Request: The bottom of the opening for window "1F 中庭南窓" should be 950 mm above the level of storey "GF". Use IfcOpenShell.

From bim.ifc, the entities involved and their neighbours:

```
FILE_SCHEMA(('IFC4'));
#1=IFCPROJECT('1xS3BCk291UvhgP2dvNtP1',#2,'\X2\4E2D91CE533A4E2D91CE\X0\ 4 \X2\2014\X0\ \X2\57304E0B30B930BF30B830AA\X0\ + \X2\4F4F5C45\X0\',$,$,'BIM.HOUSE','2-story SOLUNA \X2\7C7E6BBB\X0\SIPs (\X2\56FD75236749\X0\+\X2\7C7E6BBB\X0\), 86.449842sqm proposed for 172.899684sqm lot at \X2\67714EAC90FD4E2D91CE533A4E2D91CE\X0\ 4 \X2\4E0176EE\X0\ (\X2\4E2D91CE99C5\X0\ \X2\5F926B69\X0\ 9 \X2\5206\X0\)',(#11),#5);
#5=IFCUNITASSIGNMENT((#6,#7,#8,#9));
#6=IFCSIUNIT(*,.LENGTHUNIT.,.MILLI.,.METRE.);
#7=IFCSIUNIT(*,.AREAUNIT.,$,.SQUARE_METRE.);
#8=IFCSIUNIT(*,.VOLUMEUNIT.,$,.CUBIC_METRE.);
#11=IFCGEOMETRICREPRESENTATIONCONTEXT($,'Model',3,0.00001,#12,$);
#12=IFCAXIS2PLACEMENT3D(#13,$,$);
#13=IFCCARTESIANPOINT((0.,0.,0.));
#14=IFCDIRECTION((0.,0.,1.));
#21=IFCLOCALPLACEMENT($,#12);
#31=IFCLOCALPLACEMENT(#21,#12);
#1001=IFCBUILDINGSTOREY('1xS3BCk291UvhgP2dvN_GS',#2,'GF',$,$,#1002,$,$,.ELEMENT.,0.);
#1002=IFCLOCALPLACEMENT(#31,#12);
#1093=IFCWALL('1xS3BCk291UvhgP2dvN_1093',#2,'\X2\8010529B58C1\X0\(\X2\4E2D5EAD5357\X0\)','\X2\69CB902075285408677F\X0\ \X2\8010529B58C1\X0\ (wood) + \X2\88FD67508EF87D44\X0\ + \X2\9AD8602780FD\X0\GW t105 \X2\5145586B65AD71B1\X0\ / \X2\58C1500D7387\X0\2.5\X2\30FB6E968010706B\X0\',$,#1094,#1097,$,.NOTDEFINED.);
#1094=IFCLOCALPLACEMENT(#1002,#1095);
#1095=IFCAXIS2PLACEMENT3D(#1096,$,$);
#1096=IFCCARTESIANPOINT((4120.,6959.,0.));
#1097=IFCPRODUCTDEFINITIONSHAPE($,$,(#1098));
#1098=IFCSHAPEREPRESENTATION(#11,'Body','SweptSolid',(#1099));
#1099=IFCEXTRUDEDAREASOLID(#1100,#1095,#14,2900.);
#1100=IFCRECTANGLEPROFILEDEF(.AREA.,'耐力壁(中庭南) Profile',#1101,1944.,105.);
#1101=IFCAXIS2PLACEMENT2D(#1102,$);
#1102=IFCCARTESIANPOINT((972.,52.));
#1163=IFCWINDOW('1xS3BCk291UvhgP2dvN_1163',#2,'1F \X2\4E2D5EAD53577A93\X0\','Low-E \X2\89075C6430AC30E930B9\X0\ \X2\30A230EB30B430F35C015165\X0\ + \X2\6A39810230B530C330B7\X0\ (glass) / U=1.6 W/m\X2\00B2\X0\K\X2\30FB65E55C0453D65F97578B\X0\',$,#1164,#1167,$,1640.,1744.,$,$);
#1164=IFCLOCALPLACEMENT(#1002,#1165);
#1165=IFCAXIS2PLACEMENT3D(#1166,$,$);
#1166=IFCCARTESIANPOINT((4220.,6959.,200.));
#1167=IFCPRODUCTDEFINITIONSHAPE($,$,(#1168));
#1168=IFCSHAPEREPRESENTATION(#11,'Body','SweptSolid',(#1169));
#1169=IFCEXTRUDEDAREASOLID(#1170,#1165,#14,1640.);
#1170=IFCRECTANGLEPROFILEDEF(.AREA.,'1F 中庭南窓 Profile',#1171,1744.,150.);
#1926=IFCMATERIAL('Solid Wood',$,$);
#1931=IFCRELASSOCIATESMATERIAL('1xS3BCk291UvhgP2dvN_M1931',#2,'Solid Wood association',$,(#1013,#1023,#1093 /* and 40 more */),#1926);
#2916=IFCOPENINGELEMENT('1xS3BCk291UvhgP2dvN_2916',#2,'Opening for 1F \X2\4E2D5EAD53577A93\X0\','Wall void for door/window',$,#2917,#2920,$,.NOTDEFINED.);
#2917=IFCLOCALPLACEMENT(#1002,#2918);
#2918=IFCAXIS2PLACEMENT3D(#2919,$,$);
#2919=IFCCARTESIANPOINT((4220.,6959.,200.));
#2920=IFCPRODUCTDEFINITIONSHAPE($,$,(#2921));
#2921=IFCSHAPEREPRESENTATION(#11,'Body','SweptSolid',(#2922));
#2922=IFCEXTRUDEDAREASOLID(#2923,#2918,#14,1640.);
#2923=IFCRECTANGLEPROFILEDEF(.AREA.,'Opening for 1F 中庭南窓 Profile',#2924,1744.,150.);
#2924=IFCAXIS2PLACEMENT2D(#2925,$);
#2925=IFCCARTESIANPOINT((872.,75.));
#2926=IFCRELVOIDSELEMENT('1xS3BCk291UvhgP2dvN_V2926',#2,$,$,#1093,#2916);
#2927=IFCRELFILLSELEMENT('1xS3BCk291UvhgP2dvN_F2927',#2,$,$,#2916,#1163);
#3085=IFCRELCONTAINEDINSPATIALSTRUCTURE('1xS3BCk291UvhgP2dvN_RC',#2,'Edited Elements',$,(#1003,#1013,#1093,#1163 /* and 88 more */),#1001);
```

```python
import numpy as np
import ifcopenshell
import ifcopenshell.api.geometry
import ifcopenshell.geom
import ifcopenshell.util.element
import ifcopenshell.util.placement
import ifcopenshell.util.shape
import ifcopenshell.util.unit

model = ifcopenshell.open("bim.ifc")
unit_scale = ifcopenshell.util.unit.calculate_unit_scale(model)

window = model.by_guid("1xS3BCk291UvhgP2dvN_1163")
opening = window.FillsVoids[0].RelatingOpeningElement
storey = ifcopenshell.util.element.get_container(window, ifc_class="IfcBuildingStorey")
level = ifcopenshell.util.placement.get_local_placement(storey.ObjectPlacement)[2, 3]

# The opening's origin need not be at the sill, so measure its lowest point.
shape = ifcopenshell.geom.create_shape(ifcopenshell.geom.settings(), opening)
bottom = ifcopenshell.util.shape.get_shape_bottom_elevation(shape, shape.geometry) / unit_scale
dz = level + 0.95 / unit_scale - bottom

shift = np.array([0.0, 0.0, dz])
# The window is not placed relative to its opening, so move both.
for product in (opening, window):
    matrix = ifcopenshell.util.placement.get_local_placement(product.ObjectPlacement)
    matrix[:3, 3] += shift
    ifcopenshell.api.geometry.edit_object_placement(model, product=product, matrix=matrix, is_si=False)

print(f"moved by {dz * unit_scale:+.3f} m")

model.write("bim_updated.ifc")
```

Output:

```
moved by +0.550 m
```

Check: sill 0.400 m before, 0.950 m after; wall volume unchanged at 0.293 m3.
